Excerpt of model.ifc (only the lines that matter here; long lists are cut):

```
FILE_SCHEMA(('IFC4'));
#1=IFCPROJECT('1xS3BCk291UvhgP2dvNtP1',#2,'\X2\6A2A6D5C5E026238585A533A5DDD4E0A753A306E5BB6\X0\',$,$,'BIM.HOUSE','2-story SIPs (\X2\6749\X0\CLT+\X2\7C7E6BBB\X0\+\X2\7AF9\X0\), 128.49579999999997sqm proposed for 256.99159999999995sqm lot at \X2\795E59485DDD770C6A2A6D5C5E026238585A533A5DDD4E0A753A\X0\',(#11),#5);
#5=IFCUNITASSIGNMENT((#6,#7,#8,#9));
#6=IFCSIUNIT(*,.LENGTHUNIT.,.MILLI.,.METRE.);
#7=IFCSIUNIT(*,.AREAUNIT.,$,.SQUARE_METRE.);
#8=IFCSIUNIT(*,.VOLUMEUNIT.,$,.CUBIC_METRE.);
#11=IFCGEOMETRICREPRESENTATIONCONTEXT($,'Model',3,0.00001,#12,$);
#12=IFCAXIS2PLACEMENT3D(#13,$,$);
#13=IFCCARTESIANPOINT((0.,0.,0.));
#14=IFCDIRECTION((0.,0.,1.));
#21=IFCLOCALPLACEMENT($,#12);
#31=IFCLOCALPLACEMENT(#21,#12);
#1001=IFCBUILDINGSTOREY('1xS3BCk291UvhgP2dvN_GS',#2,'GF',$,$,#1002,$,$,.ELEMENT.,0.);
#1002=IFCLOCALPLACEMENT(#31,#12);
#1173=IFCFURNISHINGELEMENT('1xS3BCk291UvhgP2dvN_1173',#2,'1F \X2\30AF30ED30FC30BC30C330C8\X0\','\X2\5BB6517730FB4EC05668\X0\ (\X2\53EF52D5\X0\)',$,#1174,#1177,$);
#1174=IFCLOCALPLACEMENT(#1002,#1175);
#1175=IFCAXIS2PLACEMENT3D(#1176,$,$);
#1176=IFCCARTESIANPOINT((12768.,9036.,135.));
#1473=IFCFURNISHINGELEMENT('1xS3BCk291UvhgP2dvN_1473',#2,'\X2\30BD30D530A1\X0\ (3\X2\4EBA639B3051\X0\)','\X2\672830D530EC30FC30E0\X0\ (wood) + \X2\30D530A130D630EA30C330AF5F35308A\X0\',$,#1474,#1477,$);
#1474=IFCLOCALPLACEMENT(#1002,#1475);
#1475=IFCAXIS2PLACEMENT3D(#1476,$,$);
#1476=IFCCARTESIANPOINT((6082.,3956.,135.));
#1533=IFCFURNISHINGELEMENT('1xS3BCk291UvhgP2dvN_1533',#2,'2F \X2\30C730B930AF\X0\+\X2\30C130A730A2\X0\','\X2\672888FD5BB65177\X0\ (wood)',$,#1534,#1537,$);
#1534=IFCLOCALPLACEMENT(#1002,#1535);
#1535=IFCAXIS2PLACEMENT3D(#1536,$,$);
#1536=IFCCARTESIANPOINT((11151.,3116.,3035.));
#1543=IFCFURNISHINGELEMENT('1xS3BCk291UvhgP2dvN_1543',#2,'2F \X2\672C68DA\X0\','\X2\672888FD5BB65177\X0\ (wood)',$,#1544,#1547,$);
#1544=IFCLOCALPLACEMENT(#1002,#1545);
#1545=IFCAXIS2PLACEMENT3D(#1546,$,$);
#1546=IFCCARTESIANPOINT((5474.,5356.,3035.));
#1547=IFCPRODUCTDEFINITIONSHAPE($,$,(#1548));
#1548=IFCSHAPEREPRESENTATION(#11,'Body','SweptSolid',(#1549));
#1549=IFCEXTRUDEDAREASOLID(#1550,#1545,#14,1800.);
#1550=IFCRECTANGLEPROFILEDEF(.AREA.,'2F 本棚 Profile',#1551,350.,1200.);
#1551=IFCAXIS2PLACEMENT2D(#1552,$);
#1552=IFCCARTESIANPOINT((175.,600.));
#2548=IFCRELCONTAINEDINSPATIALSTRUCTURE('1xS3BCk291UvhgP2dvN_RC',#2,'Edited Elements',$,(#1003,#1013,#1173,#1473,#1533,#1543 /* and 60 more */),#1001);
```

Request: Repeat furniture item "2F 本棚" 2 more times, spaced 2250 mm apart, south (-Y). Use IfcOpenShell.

```python
import numpy as np
import ifcopenshell
import ifcopenshell.api.geometry
import ifcopenshell.api.root
import ifcopenshell.util.element
import ifcopenshell.util.placement
import ifcopenshell.util.unit

model = ifcopenshell.open("model.ifc")
unit_scale = ifcopenshell.util.unit.calculate_unit_scale(model)


def reuse_history(source, copy):
    """copy_class also copies each property set's owner history, people and application; keep the originals."""
    for rel in copy.IsDefinedBy:
        if rel.is_a("IfcRelDefinesByProperties") and (history := rel.RelatingPropertyDefinition.OwnerHistory):
            rel.RelatingPropertyDefinition.OwnerHistory = source.OwnerHistory
            ifcopenshell.util.element.remove_deep2(model, history)


source = model.by_id(1543)
base = ifcopenshell.util.placement.get_local_placement(source.ObjectPlacement)
step = np.array([0.0, -1.0, 0.0]) * 2.25 / unit_scale

for i in range(1, 3):
    copy = ifcopenshell.api.root.copy_class(model, product=source)
    copy.Representation = ifcopenshell.util.element.copy_deep(
        model, source.Representation, exclude=["IfcGeometricRepresentationContext", "IfcRepresentationMap"]
    )
    reuse_history(source, copy)
    matrix = base.copy()
    matrix[:3, 3] += i * step
    print("added at", matrix[:3, 3].round(3) + 0.0)
    ifcopenshell.api.geometry.edit_object_placement(model, product=copy, matrix=matrix, is_si=False)

model.write("model_edited.ifc")
```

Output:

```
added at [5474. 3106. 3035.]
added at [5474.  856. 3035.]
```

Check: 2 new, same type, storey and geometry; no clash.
